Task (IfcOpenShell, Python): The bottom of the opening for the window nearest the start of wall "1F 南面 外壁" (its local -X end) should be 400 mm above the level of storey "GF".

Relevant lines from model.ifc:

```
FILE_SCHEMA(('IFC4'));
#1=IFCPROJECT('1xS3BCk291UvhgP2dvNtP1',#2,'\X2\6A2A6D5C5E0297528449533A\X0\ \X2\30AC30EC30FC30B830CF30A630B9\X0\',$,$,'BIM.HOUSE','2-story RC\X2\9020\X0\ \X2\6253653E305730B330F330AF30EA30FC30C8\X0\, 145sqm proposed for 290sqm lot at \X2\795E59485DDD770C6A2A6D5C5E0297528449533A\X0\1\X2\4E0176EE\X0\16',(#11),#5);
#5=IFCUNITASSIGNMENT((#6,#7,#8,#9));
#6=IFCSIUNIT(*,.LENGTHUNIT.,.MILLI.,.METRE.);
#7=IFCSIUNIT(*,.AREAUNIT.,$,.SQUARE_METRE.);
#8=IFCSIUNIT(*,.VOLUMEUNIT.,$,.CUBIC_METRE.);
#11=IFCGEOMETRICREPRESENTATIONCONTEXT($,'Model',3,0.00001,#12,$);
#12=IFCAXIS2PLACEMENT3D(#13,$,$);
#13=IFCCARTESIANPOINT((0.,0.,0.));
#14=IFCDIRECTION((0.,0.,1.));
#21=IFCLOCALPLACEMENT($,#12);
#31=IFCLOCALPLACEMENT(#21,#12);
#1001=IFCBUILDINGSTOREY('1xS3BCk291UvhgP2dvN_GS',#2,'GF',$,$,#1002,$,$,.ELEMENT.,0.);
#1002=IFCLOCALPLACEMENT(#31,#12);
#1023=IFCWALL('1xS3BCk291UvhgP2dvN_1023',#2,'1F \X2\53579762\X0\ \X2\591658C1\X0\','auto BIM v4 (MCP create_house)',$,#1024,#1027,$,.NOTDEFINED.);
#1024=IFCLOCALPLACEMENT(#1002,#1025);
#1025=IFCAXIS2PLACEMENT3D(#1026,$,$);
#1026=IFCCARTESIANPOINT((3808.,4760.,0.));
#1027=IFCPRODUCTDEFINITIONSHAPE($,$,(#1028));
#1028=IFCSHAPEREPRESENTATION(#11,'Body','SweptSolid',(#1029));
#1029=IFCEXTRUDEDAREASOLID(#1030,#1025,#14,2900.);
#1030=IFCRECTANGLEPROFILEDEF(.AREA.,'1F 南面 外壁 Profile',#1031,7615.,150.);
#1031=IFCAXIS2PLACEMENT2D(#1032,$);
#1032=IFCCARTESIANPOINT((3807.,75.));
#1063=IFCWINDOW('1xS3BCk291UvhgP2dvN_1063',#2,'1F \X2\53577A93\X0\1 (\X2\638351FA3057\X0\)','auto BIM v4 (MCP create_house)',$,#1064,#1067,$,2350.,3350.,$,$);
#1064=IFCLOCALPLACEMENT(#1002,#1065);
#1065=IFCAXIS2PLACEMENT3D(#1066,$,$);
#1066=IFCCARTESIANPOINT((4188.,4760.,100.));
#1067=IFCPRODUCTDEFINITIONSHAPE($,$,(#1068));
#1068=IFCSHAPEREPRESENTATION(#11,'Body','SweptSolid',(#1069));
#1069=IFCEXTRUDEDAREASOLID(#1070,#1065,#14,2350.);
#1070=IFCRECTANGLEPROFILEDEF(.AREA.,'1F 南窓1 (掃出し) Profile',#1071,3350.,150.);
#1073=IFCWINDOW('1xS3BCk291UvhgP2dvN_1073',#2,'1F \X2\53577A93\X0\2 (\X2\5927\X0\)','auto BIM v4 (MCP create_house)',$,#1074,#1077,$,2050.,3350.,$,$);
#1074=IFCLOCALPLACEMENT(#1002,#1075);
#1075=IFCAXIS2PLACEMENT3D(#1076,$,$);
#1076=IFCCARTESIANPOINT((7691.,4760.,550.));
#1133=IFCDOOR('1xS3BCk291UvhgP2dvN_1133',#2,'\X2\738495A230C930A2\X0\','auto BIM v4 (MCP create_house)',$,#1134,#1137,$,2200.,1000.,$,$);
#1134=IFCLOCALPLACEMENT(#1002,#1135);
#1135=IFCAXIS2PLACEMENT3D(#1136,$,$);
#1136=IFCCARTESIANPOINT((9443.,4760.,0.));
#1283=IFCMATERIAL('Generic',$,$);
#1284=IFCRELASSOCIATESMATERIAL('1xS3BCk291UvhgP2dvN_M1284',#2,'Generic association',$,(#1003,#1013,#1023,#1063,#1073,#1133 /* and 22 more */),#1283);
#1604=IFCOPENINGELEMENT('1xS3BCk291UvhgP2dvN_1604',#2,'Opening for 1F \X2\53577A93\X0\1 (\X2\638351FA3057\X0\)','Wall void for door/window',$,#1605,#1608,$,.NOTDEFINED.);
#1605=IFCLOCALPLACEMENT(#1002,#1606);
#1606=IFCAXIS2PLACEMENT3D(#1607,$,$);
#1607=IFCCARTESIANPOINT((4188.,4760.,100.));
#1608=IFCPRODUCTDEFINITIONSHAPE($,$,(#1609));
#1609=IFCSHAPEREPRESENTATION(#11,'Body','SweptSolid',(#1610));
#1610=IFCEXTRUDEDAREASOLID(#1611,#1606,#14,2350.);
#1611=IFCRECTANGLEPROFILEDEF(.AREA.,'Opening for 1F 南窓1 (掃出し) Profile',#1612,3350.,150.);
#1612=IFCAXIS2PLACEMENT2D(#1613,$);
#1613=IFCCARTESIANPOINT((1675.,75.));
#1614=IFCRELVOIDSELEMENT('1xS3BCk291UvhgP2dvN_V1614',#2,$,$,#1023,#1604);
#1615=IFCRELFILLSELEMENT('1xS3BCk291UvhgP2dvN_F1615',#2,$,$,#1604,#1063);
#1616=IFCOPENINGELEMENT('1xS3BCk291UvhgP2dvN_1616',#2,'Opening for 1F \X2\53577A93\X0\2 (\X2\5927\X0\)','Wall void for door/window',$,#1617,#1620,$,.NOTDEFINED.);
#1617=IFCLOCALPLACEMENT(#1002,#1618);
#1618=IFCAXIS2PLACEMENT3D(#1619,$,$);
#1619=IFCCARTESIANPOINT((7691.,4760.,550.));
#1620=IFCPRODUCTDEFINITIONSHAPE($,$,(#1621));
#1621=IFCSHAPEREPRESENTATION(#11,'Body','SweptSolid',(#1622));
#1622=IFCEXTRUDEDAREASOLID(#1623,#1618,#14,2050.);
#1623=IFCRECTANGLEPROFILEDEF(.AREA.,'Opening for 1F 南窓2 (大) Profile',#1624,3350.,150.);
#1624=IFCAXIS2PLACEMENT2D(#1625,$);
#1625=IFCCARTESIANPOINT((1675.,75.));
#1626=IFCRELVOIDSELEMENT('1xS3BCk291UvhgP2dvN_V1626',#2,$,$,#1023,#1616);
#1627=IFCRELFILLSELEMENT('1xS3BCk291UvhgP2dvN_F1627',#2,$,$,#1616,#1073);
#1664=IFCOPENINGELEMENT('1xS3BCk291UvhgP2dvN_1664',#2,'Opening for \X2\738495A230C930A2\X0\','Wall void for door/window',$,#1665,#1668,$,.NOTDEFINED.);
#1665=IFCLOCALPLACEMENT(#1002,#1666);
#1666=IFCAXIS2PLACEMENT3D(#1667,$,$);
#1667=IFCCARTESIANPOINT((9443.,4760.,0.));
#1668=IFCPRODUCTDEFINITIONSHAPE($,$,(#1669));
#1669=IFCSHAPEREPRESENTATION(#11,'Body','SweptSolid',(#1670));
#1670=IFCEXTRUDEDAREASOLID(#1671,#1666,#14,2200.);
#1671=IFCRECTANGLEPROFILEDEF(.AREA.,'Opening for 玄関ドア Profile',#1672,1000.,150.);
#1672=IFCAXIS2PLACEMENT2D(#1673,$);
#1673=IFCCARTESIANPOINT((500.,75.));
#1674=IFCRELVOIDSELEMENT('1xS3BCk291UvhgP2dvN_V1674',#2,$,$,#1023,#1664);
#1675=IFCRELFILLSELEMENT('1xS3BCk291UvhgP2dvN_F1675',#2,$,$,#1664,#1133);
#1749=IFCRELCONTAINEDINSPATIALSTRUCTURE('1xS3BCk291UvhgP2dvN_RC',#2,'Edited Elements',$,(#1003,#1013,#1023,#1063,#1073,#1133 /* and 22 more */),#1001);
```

```python
import numpy as np
import ifcopenshell
import ifcopenshell.api.geometry
import ifcopenshell.geom
import ifcopenshell.util.element
import ifcopenshell.util.placement
import ifcopenshell.util.shape
import ifcopenshell.util.unit

model = ifcopenshell.open("model.ifc")
unit_scale = ifcopenshell.util.unit.calculate_unit_scale(model)

window = model.by_id(1063)
opening = window.FillsVoids[0].RelatingOpeningElement
storey = ifcopenshell.util.element.get_container(window, ifc_class="IfcBuildingStorey")
level = ifcopenshell.util.placement.get_local_placement(storey.ObjectPlacement)[2, 3]

# The opening's origin need not be at the sill, so measure its lowest point.
shape = ifcopenshell.geom.create_shape(ifcopenshell.geom.settings(), opening)
bottom = ifcopenshell.util.shape.get_shape_bottom_elevation(shape, shape.geometry) / unit_scale
dz = level + 0.4 / unit_scale - bottom

shift = np.array([0.0, 0.0, dz])
# The window is not placed relative to its opening, so move both.
for product in (opening, window):
    matrix = ifcopenshell.util.placement.get_local_placement(product.ObjectPlacement)
    matrix[:3, 3] += shift
    ifcopenshell.api.geometry.edit_object_placement(model, product=product, matrix=matrix, is_si=False)

print(f"moved by {dz * unit_scale:+.3f} m")

model.write("model-out.ifc")
```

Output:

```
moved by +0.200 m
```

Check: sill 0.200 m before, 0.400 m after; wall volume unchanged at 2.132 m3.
